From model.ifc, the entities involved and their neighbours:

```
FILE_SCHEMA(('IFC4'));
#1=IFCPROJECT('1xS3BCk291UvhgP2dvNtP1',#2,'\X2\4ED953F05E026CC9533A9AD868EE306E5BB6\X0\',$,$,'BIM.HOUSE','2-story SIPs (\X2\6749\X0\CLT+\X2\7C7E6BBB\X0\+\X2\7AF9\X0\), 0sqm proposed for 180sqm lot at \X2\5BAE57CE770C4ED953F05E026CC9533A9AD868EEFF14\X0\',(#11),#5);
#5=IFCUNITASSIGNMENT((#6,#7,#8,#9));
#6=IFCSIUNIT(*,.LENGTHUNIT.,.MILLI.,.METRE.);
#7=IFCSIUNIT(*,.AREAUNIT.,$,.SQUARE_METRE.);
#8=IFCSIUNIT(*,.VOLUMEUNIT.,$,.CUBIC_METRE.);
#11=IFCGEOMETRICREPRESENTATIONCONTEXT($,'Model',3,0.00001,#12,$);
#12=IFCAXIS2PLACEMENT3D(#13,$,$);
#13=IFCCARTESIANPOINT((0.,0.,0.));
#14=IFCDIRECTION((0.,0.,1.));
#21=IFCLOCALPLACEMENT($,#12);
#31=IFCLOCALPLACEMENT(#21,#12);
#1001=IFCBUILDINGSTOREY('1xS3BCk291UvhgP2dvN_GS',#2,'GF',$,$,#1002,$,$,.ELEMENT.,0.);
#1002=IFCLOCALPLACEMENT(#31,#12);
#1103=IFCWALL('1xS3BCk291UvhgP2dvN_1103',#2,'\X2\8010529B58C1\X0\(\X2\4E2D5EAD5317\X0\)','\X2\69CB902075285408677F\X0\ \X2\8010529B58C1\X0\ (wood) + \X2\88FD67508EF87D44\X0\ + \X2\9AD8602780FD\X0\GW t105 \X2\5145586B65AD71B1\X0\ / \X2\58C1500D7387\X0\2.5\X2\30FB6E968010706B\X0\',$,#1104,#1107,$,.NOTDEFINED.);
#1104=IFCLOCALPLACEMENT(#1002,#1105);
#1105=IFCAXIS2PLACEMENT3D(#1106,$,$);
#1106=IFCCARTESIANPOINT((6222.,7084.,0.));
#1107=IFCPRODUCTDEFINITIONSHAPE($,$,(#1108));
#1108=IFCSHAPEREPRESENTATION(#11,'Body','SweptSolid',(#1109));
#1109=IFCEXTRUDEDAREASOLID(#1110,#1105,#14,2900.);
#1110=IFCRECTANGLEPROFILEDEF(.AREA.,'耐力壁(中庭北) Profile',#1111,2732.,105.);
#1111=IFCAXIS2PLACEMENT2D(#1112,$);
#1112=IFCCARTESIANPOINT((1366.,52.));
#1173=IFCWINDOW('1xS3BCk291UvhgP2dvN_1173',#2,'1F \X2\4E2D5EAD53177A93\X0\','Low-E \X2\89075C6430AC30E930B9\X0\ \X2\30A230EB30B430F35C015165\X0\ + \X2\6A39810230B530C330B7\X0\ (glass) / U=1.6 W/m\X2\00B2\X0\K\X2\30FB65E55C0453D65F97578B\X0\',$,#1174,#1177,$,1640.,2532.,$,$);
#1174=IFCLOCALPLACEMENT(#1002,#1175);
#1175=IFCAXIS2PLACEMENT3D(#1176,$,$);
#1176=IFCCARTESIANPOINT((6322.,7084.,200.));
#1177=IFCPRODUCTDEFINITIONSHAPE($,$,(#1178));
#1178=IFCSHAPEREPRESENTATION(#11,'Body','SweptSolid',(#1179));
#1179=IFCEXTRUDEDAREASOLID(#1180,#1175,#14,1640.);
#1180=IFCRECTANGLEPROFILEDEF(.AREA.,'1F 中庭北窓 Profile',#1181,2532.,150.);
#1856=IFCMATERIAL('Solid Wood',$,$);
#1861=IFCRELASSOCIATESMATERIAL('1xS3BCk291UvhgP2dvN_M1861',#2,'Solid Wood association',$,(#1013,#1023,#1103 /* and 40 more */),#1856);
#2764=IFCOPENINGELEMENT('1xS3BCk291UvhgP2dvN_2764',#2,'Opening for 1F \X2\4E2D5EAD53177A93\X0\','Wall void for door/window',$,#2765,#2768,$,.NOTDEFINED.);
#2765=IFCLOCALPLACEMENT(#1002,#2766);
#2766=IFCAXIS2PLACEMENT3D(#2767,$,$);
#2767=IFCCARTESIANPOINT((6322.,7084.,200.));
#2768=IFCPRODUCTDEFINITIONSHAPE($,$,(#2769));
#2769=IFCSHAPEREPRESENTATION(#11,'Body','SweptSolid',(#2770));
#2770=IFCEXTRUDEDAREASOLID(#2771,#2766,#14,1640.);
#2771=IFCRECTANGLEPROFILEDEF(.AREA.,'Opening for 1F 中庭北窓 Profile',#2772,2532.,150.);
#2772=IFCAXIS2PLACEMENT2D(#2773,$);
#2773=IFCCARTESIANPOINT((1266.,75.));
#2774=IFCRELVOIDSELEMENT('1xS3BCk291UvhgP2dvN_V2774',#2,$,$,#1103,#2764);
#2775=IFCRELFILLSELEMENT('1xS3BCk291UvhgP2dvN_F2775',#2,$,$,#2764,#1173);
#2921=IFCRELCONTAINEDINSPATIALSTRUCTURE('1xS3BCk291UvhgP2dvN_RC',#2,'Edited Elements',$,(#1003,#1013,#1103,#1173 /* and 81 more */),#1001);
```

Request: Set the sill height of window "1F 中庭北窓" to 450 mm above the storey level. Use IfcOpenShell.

```python
import numpy as np
import ifcopenshell
import ifcopenshell.api.geometry
import ifcopenshell.geom
import ifcopenshell.util.element
import ifcopenshell.util.placement
import ifcopenshell.util.shape
import ifcopenshell.util.unit

model = ifcopenshell.open("model.ifc")
unit_scale = ifcopenshell.util.unit.calculate_unit_scale(model)

window = model.by_guid("1xS3BCk291UvhgP2dvN_1173")
opening = window.FillsVoids[0].RelatingOpeningElement
storey = ifcopenshell.util.element.get_container(window, ifc_class="IfcBuildingStorey")
level = ifcopenshell.util.placement.get_local_placement(storey.ObjectPlacement)[2, 3]

# The opening's origin need not be at the sill, so measure its lowest point.
shape = ifcopenshell.geom.create_shape(ifcopenshell.geom.settings(), opening)
bottom = ifcopenshell.util.shape.get_shape_bottom_elevation(shape, shape.geometry) / unit_scale
dz = level + 0.45 / unit_scale - bottom

shift = np.array([0.0, 0.0, dz])
# The window is not placed relative to its opening, so move both.
for product in (opening, window):
    matrix = ifcopenshell.util.placement.get_local_placement(product.ObjectPlacement)
    matrix[:3, 3] += shift
    ifcopenshell.api.geometry.edit_object_placement(model, product=product, matrix=matrix, is_si=False)

print(f"moved by {dz * unit_scale:+.3f} m")

model.write("model-out.ifc")
```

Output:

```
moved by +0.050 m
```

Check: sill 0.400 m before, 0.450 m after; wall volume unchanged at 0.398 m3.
